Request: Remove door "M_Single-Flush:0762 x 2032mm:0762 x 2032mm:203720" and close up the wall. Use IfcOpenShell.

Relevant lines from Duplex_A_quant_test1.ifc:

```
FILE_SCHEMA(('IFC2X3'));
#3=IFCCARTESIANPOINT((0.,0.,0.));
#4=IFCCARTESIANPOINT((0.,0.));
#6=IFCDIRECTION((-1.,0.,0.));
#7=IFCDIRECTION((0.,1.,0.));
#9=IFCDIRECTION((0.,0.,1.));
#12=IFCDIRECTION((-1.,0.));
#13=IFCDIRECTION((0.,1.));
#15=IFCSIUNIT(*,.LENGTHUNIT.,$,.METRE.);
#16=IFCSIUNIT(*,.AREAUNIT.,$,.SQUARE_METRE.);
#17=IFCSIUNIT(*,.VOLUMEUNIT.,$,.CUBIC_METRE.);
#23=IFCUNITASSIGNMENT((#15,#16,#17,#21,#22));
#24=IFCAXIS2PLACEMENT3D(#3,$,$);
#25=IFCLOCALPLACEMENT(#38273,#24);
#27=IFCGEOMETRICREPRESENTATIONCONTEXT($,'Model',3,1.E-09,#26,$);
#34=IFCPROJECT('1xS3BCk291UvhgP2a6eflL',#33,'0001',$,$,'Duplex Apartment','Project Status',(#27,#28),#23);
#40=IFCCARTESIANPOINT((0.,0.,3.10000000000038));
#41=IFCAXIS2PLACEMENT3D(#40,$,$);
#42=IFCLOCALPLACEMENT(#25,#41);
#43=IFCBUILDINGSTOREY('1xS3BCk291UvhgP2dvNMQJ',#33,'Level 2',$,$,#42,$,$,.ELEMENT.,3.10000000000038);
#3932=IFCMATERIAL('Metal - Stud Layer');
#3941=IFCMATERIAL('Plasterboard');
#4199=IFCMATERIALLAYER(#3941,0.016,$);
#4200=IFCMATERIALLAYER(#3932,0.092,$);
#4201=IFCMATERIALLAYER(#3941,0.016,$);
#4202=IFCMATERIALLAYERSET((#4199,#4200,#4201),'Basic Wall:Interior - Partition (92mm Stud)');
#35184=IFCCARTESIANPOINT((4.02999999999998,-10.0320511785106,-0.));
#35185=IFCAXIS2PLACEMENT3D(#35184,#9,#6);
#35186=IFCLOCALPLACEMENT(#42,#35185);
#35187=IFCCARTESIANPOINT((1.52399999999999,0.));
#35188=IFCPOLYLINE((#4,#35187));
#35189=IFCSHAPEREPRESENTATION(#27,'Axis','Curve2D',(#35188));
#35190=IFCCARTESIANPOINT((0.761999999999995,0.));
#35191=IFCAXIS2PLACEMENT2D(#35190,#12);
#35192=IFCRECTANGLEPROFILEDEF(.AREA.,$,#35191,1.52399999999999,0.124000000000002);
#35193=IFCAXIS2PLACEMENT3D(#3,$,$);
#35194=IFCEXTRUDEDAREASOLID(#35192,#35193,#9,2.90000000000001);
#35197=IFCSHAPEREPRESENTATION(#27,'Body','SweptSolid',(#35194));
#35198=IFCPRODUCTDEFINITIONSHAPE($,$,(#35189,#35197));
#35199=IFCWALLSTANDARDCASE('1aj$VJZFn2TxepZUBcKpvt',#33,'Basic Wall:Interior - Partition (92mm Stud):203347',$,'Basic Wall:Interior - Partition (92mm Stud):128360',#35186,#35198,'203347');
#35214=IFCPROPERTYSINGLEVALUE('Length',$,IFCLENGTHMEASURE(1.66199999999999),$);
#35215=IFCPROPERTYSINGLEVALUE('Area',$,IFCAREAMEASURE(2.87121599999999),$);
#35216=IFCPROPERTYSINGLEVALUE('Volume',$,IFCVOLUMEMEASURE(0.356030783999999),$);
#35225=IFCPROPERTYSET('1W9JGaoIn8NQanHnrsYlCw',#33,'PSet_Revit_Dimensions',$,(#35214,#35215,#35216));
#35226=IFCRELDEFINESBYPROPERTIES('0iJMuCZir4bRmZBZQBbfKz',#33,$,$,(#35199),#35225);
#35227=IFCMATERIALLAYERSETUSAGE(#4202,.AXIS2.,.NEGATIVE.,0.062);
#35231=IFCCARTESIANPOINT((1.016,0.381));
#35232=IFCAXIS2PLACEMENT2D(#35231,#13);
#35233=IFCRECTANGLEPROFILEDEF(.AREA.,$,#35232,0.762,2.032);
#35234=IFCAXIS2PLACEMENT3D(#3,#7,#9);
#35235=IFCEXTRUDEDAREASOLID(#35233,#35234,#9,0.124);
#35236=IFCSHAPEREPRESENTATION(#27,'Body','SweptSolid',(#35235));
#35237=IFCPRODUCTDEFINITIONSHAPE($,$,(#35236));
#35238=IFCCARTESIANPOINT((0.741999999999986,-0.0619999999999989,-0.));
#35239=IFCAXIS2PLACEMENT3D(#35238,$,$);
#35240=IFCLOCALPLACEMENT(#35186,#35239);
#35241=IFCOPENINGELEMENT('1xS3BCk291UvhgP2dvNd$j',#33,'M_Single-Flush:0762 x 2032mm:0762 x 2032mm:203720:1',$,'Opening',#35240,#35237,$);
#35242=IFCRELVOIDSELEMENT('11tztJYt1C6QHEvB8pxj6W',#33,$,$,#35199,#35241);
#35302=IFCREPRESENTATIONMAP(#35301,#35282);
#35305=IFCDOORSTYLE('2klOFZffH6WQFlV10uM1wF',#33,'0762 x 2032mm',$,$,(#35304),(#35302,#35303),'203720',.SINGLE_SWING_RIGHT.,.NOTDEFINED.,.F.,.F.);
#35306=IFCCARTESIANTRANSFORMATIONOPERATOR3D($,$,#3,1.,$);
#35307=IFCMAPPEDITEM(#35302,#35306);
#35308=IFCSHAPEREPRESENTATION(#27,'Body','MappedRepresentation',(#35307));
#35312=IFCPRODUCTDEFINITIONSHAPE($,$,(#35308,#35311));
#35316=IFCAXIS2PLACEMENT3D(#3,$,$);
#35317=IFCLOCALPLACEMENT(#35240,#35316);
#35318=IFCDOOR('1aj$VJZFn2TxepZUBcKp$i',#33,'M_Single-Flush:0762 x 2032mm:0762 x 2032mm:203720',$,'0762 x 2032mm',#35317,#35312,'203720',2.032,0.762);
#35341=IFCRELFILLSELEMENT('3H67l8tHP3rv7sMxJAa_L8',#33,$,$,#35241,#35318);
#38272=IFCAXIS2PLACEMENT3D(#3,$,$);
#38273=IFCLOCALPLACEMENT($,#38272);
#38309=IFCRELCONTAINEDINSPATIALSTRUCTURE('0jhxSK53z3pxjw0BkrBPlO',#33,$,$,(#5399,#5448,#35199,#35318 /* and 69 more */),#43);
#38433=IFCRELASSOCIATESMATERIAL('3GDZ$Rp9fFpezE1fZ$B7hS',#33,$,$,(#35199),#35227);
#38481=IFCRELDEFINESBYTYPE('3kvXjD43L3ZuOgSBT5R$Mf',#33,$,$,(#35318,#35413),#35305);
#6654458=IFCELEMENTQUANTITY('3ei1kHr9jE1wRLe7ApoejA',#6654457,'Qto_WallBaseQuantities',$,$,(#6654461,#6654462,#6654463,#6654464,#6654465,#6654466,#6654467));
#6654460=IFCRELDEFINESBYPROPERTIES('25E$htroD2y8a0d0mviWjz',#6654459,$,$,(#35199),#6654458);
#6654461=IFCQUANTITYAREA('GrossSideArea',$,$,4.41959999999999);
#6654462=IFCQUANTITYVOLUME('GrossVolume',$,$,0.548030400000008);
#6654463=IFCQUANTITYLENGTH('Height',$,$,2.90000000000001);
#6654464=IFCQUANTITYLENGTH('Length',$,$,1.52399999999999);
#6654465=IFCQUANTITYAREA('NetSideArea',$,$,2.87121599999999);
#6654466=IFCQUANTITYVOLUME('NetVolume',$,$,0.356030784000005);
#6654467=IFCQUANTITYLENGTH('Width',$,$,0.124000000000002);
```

```python
import ifcopenshell
import ifcopenshell.api.feature
import ifcopenshell.api.pset
import ifcopenshell.api.root
import ifcopenshell.geom
import ifcopenshell.util.element
import ifcopenshell.util.shape
import ifcopenshell.util.unit

model = ifcopenshell.open("Duplex_A_quant_test1.ifc")
area_scale = ifcopenshell.util.unit.calculate_unit_scale(model, "AREAUNIT")
volume_scale = ifcopenshell.util.unit.calculate_unit_scale(model, "VOLUMEUNIT")
settings = ifcopenshell.geom.settings()


def volume(element):
    """Net volume in cubic metres, openings subtracted."""
    shape = ifcopenshell.geom.create_shape(settings, element)
    return ifcopenshell.util.shape.get_volume(shape.geometry)


door = model.by_guid("1aj$VJZFn2TxepZUBcKp$i")
opening = door.FillsVoids[0].RelatingOpeningElement
wall = opening.VoidsElements[0].RelatingBuildingElement
before = volume(wall)

ifcopenshell.api.root.remove_product(model, product=door)
ifcopenshell.api.feature.remove_feature(model, feature=opening)

after = volume(wall)
thickness = 0.124  # wall thickness in metres

# Update the wall's stored quantities.
pset = model.by_id(ifcopenshell.util.element.get_pset(wall, "PSet_Revit_Dimensions", should_inherit=False)["id"])
ifcopenshell.api.pset.edit_pset(model, pset=pset, properties={
    "Area": model.create_entity("IfcAreaMeasure", after / thickness / area_scale),
    "Volume": model.create_entity("IfcVolumeMeasure", after / volume_scale),
})
qto = model.by_id(ifcopenshell.util.element.get_pset(wall, "Qto_WallBaseQuantities", should_inherit=False)["id"])
ifcopenshell.api.pset.edit_qto(model, qto=qto, properties={
    "NetSideArea": after / thickness / area_scale,
    "NetVolume": after / volume_scale,
})

print(f"wall volume {before:.3f} -> {after:.3f} m3")

model.write("Duplex_A_quant_test1_updated.ifc")
```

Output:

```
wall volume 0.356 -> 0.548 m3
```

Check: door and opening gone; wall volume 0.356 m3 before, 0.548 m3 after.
